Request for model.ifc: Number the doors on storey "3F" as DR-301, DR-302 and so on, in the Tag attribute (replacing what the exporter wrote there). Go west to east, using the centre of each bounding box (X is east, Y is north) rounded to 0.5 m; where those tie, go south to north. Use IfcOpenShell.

First a look at what the model holds.

```python
import ifcopenshell
import ifcopenshell.util.element
import ifcopenshell.util.placement

model = ifcopenshell.open("model.ifc")
print(model.schema)
storey = next(s for s in model.by_type("IfcBuildingStorey") if s.Name == "3F")
doors = [e for e in ifcopenshell.util.element.get_decomposition(storey) if e.is_a("IfcDoor")]
for e in sorted(doors, key=lambda e: e.id()):
    origin = ifcopenshell.util.placement.get_local_placement(e.ObjectPlacement)[:3, 3]
    print(e.id(), e.Tag, e.Name, origin.round(2) + 0.0, sep=" | ")
```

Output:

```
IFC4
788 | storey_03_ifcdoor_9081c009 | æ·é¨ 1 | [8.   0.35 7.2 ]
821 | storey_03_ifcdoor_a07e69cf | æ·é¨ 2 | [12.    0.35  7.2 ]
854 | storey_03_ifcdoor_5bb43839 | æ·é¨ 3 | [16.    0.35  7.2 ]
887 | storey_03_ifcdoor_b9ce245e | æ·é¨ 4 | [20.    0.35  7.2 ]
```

```python
import ifcopenshell
import ifcopenshell.geom
import ifcopenshell.util.element
import ifcopenshell.util.shape

model = ifcopenshell.open("model.ifc")
settings = ifcopenshell.geom.settings()
settings.set("use-world-coords", True)


def centre(element):
    shape = ifcopenshell.geom.create_shape(settings, element)
    return ifcopenshell.util.shape.get_bbox_centroid(shape.geometry)


storey = next(s for s in model.by_type("IfcBuildingStorey") if s.Name == "3F")
doors = [e for e in ifcopenshell.util.element.get_decomposition(storey) if e.is_a("IfcDoor")]

# Insertion points can sit at a corner or the storey origin, so sort by the geometry (in metres).
centres = {e: centre(e) for e in doors}
doors.sort(key=lambda e: (round(centres[e][0] / 0.5), centres[e][1]))

for i, e in enumerate(doors, start=1):
    number = f"DR-3{i:02d}"
    e.Tag = number
    print(e.id(), number)

model.write("model-out.ifc")
```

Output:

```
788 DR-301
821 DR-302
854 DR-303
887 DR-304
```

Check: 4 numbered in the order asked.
